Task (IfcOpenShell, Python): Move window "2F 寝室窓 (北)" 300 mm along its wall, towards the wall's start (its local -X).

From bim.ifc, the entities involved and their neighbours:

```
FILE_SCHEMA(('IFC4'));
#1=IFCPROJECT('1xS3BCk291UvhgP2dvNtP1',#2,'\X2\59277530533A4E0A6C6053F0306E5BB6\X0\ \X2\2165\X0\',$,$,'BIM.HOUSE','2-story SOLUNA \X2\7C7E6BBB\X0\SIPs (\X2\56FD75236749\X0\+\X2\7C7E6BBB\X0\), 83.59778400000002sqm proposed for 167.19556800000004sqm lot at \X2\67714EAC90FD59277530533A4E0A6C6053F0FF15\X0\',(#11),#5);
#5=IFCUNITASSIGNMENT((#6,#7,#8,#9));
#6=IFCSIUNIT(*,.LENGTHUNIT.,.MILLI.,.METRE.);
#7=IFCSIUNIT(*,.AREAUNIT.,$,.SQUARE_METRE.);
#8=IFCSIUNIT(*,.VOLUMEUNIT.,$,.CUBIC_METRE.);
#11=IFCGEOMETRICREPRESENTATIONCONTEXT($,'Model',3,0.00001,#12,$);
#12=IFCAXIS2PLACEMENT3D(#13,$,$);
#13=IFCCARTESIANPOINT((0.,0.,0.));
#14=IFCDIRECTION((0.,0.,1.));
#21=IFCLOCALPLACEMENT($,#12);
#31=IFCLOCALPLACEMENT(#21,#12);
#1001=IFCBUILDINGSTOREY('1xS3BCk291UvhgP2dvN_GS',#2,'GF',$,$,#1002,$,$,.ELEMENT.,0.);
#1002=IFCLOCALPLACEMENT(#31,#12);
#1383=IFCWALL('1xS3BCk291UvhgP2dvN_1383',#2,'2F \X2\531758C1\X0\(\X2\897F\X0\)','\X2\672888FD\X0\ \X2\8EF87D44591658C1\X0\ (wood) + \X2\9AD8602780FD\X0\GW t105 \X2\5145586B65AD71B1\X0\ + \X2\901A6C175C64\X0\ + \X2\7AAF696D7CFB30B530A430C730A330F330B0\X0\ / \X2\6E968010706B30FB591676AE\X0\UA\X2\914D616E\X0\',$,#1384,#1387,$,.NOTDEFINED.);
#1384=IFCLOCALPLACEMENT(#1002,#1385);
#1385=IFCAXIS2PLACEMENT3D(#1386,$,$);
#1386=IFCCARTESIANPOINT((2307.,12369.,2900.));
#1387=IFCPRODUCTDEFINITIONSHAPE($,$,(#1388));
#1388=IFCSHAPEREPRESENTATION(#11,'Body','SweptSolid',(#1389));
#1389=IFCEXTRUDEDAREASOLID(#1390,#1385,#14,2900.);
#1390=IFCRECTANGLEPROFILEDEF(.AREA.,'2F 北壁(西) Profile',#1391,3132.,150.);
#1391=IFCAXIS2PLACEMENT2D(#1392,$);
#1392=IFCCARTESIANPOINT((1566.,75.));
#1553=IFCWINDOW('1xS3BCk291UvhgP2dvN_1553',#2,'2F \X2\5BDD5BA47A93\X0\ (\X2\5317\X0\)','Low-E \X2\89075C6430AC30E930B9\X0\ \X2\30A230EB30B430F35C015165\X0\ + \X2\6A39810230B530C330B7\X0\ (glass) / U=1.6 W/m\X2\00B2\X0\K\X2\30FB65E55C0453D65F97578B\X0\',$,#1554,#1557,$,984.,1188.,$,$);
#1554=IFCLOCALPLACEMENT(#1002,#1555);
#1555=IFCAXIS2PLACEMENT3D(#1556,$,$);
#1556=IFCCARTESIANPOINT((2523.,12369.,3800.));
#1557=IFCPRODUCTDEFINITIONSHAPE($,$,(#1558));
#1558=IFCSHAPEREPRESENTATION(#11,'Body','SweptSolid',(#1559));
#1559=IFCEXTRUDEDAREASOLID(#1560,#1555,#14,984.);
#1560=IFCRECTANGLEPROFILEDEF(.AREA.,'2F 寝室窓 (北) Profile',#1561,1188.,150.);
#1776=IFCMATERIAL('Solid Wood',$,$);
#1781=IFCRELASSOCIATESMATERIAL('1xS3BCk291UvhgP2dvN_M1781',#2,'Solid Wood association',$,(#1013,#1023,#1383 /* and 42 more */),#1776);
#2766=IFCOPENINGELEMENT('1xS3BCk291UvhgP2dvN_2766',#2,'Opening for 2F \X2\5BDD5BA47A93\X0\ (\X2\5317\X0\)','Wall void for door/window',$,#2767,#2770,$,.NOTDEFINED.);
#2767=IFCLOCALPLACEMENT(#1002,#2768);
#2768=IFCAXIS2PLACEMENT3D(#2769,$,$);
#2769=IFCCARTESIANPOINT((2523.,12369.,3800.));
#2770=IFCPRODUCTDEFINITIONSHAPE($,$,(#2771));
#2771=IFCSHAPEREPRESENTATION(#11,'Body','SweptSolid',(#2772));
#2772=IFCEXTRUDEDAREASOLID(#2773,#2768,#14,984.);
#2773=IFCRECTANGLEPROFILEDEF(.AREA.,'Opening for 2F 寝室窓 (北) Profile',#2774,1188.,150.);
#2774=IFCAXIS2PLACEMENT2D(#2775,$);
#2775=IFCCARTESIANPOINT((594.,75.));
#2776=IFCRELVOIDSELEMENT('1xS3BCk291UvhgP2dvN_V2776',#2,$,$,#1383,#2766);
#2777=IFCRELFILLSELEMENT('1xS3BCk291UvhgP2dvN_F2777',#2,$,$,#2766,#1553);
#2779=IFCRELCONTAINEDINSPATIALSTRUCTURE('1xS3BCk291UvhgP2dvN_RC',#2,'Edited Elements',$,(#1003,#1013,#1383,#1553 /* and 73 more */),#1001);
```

```python
import ifcopenshell
import ifcopenshell.api.geometry
import ifcopenshell.util.placement
import ifcopenshell.util.unit

model = ifcopenshell.open("bim.ifc")
unit_scale = ifcopenshell.util.unit.calculate_unit_scale(model)

window = model.by_id(1553)
opening = window.FillsVoids[0].RelatingOpeningElement
wall = opening.VoidsElements[0].RelatingBuildingElement

wall_matrix = ifcopenshell.util.placement.get_local_placement(wall.ObjectPlacement)
shift = wall_matrix[:3, 0] * -0.3 / unit_scale
before = ifcopenshell.util.placement.get_local_placement(window.ObjectPlacement)[:3, 3].copy()

# The window is not placed relative to its opening, so move both.
for product in (opening, window):
    matrix = ifcopenshell.util.placement.get_local_placement(product.ObjectPlacement)
    matrix[:3, 3] += shift
    ifcopenshell.api.geometry.edit_object_placement(model, product=product, matrix=matrix, is_si=False)

after = ifcopenshell.util.placement.get_local_placement(window.ObjectPlacement)[:3, 3]
print("window moved by", (after - before).round(3) + 0.0)

model.write("bim_updated.ifc")
```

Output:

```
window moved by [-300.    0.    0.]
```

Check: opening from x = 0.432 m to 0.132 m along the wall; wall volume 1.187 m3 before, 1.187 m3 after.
